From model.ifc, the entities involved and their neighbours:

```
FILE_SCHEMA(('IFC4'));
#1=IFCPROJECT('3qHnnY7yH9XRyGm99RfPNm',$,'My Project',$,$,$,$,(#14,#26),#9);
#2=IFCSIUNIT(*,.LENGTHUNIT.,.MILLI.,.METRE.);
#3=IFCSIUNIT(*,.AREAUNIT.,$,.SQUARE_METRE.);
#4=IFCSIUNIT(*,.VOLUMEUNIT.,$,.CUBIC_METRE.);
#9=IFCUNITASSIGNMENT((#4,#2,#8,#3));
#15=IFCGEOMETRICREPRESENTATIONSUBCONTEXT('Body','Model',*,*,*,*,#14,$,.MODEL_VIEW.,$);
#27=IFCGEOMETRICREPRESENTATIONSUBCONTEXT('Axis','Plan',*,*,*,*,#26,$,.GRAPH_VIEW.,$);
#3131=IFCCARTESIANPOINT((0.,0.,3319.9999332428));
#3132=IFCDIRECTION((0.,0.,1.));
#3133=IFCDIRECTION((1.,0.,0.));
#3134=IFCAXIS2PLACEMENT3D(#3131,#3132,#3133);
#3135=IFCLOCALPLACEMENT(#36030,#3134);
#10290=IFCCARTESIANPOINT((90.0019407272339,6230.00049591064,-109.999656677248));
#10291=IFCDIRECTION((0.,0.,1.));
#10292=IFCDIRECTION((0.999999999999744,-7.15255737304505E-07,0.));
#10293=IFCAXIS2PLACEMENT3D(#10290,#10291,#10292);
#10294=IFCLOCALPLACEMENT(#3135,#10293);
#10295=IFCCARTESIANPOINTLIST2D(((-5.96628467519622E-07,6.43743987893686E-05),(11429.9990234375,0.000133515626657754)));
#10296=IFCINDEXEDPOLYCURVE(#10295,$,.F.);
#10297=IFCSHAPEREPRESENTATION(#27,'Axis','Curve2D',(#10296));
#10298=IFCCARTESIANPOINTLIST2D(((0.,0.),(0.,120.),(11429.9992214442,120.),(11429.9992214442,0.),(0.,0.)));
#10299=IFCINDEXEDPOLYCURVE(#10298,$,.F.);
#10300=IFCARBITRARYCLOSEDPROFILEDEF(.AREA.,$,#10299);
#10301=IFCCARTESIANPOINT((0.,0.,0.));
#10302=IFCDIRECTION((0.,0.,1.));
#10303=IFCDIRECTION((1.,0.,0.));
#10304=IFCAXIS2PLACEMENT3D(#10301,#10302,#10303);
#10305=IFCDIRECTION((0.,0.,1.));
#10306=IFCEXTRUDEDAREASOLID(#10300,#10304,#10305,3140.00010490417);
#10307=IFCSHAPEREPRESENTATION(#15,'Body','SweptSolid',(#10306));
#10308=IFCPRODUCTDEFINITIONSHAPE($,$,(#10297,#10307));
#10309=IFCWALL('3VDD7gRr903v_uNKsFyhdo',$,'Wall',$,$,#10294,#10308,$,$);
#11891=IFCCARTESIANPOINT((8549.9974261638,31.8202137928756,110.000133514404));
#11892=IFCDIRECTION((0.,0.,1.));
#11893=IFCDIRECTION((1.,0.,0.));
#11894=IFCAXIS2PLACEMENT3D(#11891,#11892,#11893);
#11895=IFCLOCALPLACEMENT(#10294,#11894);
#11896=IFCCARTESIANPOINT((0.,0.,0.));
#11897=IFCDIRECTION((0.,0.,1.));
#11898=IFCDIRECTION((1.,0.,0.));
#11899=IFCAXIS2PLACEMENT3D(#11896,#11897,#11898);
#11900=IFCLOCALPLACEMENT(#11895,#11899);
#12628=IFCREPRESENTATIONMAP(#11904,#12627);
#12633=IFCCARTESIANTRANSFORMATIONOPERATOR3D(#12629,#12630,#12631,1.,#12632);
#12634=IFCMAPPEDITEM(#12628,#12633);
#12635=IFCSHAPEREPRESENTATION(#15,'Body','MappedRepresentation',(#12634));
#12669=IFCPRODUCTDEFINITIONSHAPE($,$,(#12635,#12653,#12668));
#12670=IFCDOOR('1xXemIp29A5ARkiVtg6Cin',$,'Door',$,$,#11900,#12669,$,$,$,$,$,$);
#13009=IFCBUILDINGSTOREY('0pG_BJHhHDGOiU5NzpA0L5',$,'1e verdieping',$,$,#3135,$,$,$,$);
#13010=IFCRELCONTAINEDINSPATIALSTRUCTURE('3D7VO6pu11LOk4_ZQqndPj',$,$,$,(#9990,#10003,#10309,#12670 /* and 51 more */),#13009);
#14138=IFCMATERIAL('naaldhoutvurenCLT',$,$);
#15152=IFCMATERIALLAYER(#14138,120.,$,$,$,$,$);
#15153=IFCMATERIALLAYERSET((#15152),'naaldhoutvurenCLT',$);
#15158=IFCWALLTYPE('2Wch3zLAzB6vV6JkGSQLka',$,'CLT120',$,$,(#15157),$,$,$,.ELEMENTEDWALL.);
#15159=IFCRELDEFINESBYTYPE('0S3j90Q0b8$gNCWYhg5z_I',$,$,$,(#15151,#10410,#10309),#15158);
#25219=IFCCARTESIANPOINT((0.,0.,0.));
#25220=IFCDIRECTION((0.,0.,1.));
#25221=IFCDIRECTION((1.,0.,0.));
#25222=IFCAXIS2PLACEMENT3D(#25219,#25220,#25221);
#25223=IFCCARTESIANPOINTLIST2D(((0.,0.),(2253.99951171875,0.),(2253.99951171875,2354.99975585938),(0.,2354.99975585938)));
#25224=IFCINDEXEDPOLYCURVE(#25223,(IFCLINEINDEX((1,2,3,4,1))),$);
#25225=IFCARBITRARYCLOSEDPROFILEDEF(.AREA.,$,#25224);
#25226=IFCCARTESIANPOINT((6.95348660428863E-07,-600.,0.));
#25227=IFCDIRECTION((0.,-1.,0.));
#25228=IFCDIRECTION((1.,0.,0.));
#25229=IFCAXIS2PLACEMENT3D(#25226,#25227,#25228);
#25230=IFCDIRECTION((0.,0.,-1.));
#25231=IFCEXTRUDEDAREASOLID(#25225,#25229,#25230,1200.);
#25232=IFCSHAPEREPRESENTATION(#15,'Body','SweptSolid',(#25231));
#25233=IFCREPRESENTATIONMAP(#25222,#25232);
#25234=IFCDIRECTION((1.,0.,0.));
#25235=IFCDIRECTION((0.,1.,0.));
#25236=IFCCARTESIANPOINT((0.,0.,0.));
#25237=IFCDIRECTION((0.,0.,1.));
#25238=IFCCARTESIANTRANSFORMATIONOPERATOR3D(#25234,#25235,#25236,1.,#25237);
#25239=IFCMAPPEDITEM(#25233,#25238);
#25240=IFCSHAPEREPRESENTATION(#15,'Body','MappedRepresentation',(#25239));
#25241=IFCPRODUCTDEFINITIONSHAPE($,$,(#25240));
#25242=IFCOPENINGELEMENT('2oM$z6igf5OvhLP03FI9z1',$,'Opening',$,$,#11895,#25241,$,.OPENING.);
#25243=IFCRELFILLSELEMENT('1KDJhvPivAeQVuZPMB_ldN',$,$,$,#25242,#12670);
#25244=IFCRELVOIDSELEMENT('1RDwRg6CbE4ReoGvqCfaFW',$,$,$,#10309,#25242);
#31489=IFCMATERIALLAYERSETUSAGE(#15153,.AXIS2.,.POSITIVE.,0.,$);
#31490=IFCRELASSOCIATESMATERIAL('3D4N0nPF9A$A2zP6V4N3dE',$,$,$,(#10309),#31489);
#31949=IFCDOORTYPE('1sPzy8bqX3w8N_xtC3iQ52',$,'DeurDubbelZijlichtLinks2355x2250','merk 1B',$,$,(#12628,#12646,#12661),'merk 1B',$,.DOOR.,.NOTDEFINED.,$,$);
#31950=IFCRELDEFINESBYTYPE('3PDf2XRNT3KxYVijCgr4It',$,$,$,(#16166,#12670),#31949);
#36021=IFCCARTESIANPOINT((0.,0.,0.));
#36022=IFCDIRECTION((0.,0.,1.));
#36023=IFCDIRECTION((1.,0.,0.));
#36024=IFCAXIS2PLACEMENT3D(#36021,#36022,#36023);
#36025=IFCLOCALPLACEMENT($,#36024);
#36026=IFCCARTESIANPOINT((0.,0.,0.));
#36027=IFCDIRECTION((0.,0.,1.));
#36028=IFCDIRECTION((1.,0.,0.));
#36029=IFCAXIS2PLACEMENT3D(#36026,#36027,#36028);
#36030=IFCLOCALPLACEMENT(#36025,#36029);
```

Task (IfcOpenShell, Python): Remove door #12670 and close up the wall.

```python
import ifcopenshell
import ifcopenshell.api.feature
import ifcopenshell.api.root
import ifcopenshell.geom
import ifcopenshell.util.shape

model = ifcopenshell.open("model.ifc")
settings = ifcopenshell.geom.settings()


def volume(element):
    """Net volume in cubic metres, openings subtracted."""
    shape = ifcopenshell.geom.create_shape(settings, element)
    return ifcopenshell.util.shape.get_volume(shape.geometry)


door = model.by_guid("1xXemIp29A5ARkiVtg6Cin")
opening = door.FillsVoids[0].RelatingOpeningElement
wall = opening.VoidsElements[0].RelatingBuildingElement
before = volume(wall)

ifcopenshell.api.root.remove_product(model, product=door)
ifcopenshell.api.feature.remove_feature(model, feature=opening)

after = volume(wall)

print(f"wall volume {before:.3f} -> {after:.3f} m3")

model.write("model_edited.ifc")
```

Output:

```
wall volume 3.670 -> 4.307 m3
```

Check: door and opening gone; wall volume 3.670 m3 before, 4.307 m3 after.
